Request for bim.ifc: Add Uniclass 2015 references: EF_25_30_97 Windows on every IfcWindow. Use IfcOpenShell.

First a look at what the model holds.

```python
import ifcopenshell

model = ifcopenshell.open("bim.ifc")
print(model.schema)
print("classifications:", [c.Name for c in model.by_type("IfcClassification")])
for ifc_class in ("IfcDoor", "IfcRoof", "IfcStair", "IfcWall", "IfcWindow"):
    print(ifc_class, len(model.by_type(ifc_class)))
```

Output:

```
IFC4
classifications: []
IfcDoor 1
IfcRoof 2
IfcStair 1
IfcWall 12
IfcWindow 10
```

```python
import ifcopenshell
import ifcopenshell.api.classification

model = ifcopenshell.open("bim.ifc")

system = ifcopenshell.api.classification.add_classification(model, classification="Uniclass 2015")

codes = {
    "IfcWindow": ("EF_25_30_97", "Windows"),
}
for ifc_class, (code, name) in codes.items():
    products = model.by_type(ifc_class)
    ifcopenshell.api.classification.add_reference(
        model, products=products, classification=system, identification=code, name=name
    )
    print(code, len(products))

model.write("bim_updated.ifc")
```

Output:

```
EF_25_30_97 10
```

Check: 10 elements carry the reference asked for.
